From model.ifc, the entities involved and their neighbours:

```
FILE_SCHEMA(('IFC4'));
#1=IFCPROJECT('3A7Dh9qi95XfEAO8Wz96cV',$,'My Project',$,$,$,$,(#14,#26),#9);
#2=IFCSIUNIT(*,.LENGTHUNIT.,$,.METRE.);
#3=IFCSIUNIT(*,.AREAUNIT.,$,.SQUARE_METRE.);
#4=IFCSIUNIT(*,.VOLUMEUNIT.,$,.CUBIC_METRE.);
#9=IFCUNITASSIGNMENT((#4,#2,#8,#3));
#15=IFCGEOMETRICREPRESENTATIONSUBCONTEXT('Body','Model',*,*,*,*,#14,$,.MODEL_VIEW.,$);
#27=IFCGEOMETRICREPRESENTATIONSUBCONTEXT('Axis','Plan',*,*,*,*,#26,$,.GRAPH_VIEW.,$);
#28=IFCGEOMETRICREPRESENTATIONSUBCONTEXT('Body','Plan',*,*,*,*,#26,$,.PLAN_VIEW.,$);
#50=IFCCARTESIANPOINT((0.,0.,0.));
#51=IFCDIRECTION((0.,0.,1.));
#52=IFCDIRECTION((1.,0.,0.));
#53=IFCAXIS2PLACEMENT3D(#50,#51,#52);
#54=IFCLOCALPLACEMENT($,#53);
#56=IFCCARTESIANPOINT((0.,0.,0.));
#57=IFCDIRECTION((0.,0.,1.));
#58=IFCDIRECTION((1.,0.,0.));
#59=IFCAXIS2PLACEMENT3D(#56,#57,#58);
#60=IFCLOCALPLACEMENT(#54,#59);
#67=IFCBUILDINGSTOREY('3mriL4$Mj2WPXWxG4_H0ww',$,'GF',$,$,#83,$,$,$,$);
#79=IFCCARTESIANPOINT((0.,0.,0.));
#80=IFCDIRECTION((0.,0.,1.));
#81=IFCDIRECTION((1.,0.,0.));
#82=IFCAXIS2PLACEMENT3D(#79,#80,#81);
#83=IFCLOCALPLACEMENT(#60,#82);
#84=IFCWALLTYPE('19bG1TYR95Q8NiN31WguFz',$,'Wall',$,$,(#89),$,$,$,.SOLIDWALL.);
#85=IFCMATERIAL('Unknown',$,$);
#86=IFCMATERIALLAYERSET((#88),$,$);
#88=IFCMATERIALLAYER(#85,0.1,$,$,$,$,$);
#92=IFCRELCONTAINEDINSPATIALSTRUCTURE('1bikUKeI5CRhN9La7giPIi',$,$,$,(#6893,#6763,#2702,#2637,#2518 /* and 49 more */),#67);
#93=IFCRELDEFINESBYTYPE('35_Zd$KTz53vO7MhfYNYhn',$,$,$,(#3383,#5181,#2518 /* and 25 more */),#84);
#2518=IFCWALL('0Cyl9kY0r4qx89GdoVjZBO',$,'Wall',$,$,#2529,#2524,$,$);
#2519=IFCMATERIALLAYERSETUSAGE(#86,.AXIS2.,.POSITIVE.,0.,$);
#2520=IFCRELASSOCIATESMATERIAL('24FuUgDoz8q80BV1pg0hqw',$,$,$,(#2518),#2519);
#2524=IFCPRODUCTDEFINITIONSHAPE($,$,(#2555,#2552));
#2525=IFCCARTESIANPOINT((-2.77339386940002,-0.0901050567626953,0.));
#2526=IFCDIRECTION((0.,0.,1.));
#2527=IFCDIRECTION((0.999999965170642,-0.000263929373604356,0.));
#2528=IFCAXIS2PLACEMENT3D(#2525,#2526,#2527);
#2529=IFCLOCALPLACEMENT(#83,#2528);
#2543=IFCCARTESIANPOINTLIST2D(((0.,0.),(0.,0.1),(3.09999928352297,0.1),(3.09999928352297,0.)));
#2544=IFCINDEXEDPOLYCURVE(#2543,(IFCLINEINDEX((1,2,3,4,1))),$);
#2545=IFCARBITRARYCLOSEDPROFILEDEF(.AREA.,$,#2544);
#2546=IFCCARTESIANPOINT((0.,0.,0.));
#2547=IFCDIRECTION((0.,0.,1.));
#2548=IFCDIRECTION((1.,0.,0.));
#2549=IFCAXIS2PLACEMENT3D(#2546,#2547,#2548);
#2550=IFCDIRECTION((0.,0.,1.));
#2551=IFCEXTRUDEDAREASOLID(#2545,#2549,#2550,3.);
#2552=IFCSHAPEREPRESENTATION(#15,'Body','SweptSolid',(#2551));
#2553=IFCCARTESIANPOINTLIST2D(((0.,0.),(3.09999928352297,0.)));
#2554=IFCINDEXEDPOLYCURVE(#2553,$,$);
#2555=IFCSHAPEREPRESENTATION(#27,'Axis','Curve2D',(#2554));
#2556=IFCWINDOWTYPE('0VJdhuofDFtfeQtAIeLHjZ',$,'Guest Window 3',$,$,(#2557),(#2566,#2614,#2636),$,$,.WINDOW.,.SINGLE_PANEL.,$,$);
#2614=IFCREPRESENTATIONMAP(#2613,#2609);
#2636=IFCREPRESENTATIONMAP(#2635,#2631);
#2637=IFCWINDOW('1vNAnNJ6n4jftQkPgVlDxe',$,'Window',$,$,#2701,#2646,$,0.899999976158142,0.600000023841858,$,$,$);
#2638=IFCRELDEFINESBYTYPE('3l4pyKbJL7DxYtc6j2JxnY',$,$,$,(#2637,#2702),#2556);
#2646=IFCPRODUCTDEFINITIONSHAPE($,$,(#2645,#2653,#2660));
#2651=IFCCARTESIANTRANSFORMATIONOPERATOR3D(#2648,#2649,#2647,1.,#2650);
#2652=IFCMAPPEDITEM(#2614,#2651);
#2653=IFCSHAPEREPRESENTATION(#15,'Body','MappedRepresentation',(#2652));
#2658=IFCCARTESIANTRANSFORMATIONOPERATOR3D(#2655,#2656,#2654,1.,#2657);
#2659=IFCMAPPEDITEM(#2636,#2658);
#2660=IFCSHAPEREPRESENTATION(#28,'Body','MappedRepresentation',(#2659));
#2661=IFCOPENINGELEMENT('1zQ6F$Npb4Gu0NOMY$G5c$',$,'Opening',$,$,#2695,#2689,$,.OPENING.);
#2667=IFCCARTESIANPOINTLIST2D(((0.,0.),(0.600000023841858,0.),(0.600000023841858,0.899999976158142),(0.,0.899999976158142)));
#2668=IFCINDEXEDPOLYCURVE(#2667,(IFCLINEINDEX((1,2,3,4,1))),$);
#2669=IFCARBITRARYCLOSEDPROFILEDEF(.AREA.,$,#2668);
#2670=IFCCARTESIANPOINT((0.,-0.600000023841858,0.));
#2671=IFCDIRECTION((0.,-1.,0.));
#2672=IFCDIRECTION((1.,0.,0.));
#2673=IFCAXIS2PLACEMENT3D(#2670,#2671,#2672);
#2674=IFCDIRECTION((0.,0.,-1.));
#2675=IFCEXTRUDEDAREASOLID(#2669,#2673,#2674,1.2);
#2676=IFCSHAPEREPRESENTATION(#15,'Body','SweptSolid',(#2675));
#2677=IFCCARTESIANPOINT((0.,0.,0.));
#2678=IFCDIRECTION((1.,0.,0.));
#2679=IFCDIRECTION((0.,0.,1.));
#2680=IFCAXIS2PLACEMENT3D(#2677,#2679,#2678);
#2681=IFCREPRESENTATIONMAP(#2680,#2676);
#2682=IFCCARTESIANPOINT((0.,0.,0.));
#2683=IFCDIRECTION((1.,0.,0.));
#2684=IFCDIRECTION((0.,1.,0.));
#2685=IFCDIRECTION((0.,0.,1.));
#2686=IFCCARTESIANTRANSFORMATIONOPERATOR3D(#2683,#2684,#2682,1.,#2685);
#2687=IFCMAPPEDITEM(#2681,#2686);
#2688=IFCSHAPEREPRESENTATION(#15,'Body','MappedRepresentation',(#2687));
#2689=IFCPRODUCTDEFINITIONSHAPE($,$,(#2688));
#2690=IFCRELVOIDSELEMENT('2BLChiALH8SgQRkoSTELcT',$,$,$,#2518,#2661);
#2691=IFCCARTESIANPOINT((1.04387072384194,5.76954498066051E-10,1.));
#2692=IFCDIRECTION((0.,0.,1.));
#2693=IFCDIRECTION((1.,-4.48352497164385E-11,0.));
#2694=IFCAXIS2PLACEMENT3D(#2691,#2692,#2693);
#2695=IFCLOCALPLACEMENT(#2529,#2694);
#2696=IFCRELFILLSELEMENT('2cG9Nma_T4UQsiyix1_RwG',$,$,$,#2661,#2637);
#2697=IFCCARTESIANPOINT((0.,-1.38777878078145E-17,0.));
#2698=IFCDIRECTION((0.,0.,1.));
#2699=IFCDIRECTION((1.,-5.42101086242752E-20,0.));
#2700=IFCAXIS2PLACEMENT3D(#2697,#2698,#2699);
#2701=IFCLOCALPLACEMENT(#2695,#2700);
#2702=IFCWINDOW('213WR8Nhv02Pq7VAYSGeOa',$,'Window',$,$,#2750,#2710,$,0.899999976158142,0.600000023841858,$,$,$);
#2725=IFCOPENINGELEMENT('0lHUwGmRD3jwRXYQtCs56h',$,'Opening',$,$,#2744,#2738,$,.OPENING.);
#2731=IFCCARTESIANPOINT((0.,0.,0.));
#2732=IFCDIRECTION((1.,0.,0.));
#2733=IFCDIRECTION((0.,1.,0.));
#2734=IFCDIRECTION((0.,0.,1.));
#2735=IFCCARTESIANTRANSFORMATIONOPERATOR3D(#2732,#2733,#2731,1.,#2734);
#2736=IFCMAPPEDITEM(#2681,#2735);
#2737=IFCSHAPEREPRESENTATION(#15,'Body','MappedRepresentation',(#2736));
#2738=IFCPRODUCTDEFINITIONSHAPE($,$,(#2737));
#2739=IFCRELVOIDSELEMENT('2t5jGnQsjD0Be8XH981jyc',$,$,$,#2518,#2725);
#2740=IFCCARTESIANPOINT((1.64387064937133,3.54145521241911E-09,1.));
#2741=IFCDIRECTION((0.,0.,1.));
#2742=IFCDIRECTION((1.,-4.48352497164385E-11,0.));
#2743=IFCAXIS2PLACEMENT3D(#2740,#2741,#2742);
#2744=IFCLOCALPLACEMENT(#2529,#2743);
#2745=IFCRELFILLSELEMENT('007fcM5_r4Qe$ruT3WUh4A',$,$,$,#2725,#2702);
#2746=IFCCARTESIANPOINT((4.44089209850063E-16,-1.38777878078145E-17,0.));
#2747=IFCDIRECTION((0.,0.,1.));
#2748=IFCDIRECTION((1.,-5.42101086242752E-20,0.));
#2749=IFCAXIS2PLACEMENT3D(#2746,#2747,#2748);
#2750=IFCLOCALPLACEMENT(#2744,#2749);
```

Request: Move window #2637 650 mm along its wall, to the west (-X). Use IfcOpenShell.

```python
import ifcopenshell
import ifcopenshell.api.geometry
import ifcopenshell.util.placement

model = ifcopenshell.open("model.ifc")

window = model.by_guid("1vNAnNJ6n4jftQkPgVlDxe")
opening = window.FillsVoids[0].RelatingOpeningElement
wall = opening.VoidsElements[0].RelatingBuildingElement

wall_matrix = ifcopenshell.util.placement.get_local_placement(wall.ObjectPlacement)
shift = wall_matrix[:3, 0] * -0.65
before = ifcopenshell.util.placement.get_local_placement(window.ObjectPlacement)[:3, 3].copy()

# The window is placed relative to its opening, so it follows when the opening moves.
matrix = ifcopenshell.util.placement.get_local_placement(opening.ObjectPlacement)
matrix[:3, 3] += shift
ifcopenshell.api.geometry.edit_object_placement(
    model, product=opening, matrix=matrix, is_si=False, should_transform_children=True
)

after = ifcopenshell.util.placement.get_local_placement(window.ObjectPlacement)[:3, 3]
print("window moved by", (after - before).round(3) + 0.0)

model.write("model-out.ifc")
```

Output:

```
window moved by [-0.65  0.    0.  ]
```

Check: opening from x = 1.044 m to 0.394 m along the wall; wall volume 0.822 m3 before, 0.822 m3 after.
